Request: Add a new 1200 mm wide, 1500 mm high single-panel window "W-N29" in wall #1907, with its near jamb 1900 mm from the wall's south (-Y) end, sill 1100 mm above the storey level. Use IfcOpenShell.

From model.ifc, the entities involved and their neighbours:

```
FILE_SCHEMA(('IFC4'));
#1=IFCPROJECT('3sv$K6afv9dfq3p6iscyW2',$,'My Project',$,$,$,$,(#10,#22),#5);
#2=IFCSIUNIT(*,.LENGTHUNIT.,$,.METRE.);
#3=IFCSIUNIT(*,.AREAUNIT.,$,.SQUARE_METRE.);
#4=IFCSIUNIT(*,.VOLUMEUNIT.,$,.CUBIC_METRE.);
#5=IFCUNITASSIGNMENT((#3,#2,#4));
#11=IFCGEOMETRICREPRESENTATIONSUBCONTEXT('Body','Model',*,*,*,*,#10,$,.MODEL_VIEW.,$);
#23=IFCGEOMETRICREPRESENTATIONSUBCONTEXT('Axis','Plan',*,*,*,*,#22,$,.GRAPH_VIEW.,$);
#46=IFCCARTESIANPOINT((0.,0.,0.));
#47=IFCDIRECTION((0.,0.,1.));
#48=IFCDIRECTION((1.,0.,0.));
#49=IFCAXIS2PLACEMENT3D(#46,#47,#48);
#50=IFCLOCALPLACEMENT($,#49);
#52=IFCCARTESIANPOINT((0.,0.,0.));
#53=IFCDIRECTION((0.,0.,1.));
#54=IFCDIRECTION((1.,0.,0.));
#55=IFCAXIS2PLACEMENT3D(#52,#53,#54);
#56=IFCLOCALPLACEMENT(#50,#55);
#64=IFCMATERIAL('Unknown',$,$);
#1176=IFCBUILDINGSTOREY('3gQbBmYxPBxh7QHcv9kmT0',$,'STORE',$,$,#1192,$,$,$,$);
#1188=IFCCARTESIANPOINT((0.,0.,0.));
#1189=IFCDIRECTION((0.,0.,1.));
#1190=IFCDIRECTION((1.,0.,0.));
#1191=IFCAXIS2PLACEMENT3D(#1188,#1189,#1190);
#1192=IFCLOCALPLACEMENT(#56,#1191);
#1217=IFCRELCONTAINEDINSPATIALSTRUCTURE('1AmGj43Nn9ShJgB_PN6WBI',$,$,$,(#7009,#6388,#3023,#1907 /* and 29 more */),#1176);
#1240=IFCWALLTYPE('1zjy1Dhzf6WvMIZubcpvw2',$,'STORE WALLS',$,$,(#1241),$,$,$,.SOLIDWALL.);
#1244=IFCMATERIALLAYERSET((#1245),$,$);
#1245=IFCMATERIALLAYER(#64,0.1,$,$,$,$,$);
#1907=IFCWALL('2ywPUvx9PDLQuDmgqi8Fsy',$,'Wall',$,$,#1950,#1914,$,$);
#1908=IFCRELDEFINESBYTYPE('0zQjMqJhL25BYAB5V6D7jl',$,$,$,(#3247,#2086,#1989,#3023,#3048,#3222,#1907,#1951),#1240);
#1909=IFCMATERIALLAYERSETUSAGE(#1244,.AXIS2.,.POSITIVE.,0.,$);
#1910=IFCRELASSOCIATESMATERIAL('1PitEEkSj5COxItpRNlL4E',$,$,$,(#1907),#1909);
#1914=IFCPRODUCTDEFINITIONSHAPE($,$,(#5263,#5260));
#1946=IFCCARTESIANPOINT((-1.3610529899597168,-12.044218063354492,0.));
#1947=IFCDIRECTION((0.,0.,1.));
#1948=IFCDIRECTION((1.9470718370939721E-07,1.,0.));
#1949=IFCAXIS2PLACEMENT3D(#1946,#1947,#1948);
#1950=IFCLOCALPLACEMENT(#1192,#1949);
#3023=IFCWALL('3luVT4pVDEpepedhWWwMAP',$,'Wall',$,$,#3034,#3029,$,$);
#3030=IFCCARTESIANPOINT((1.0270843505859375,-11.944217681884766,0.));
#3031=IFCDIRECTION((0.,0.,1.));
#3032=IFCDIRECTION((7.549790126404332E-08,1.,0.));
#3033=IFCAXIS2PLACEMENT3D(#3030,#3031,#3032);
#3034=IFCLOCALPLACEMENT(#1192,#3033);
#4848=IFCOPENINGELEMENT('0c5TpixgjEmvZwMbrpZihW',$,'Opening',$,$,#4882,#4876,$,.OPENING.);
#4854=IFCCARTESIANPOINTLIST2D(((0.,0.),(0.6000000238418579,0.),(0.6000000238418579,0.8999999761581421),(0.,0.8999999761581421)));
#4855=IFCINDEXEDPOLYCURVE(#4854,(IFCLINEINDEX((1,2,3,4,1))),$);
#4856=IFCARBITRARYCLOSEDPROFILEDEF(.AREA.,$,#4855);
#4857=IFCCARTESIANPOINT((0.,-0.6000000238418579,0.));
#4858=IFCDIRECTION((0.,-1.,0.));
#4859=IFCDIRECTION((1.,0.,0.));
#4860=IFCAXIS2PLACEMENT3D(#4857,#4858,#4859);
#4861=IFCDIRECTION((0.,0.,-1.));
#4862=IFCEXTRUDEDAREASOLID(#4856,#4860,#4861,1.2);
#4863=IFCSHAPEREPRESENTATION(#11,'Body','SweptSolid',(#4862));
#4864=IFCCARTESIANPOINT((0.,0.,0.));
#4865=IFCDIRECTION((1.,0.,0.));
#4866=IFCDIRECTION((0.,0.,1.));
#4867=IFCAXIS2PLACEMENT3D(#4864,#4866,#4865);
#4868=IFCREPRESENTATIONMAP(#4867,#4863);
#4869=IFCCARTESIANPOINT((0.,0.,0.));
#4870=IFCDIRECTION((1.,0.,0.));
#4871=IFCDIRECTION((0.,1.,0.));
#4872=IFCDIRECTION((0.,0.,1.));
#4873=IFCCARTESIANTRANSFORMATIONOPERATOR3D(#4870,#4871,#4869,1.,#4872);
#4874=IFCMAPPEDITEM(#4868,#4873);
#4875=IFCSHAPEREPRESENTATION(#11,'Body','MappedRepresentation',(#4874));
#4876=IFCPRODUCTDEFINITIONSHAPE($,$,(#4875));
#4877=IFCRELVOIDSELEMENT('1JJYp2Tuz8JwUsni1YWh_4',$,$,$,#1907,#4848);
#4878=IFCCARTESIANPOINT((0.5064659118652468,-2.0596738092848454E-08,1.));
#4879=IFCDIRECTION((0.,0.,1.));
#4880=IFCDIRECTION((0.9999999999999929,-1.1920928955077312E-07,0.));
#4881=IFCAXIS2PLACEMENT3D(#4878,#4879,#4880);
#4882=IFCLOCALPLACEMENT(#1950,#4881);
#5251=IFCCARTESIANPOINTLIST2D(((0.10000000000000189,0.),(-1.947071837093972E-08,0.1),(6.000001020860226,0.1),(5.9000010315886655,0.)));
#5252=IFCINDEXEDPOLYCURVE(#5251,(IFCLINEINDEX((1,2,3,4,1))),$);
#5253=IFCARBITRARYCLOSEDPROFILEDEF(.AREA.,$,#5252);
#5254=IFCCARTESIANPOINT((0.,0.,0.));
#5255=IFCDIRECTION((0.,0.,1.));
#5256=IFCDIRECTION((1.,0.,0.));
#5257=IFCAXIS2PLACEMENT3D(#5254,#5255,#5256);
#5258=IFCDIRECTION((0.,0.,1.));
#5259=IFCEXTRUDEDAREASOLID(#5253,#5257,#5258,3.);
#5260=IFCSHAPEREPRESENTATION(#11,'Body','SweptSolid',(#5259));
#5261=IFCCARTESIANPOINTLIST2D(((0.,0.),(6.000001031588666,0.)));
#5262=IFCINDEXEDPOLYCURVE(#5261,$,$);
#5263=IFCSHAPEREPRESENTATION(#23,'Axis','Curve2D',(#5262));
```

```python
import numpy as np
import ifcopenshell
import ifcopenshell.api.feature
import ifcopenshell.api.geometry
import ifcopenshell.api.root
import ifcopenshell.api.spatial
import ifcopenshell.geom
import ifcopenshell.util.element
import ifcopenshell.util.placement
import ifcopenshell.util.representation
import ifcopenshell.util.shape
import ifcopenshell.util.unit

model = ifcopenshell.open("model.ifc")
unit_scale = ifcopenshell.util.unit.calculate_unit_scale(model)
settings = ifcopenshell.geom.settings()


def volume(element):
    """Net volume in cubic metres, openings subtracted."""
    shape = ifcopenshell.geom.create_shape(settings, element)
    return ifcopenshell.util.shape.get_volume(shape.geometry)


wall = model.by_guid("2ywPUvx9PDLQuDmgqi8Fsy")
storey = ifcopenshell.util.element.get_container(wall, ifc_class="IfcBuildingStorey")
context = ifcopenshell.util.representation.get_context(model, "Model", "Body", "MODEL_VIEW")
before = volume(wall)

width, height, from_end, sill = 1.2, 1.5, 1.9, 1.1  # metres

# The wall runs along its own X axis, and the end named is its -X end.
wall_shape = ifcopenshell.geom.create_shape(settings, wall)
x, y, z = ifcopenshell.util.shape.get_vertices(wall_shape.geometry).T
start = x.min() + from_end
face, thickness = float(y.min()), float(y.max() - y.min())
wall_matrix = ifcopenshell.util.placement.get_local_placement(wall.ObjectPlacement)
level = ifcopenshell.util.placement.get_local_placement(storey.ObjectPlacement)[2, 3]


def in_wall(x, y):
    """Placement at x, y metres in the wall's axes, at sill height."""
    matrix = wall_matrix.copy()
    matrix[:, 3] = wall_matrix @ np.array([x / unit_scale, y / unit_scale, 0.0, 1.0])
    matrix[2, 3] = level + sill / unit_scale
    return matrix


# Opening: a box that overshoots both wall faces by 50 mm.
opening = ifcopenshell.api.root.create_entity(model, ifc_class="IfcOpeningElement", predefined_type="OPENING")
box = ifcopenshell.api.geometry.add_wall_representation(
    model, context=context, length=width, height=height, thickness=thickness + 0.1
)
ifcopenshell.api.geometry.assign_representation(model, product=opening, representation=box)
ifcopenshell.api.geometry.edit_object_placement(model, product=opening, matrix=in_wall(start, face - 0.05), is_si=False)
ifcopenshell.api.feature.add_feature(model, feature=opening, element=wall)

window = ifcopenshell.api.root.create_entity(model, ifc_class="IfcWindow", name="W-N29", predefined_type="WINDOW")
window.OverallWidth, window.OverallHeight = width / unit_scale, height / unit_scale
window.PartitioningType = "SINGLE_PANEL"
body = ifcopenshell.api.geometry.add_window_representation(
    model,
    context=context,
    overall_width=window.OverallWidth,
    overall_height=window.OverallHeight,
    partition_type="SINGLE_PANEL",
)
ifcopenshell.api.geometry.assign_representation(model, product=window, representation=body)
ifcopenshell.api.spatial.assign_container(model, products=[window], relating_structure=storey)
ifcopenshell.api.feature.add_filling(model, opening=opening, element=window)

# Centre the window in the wall's thickness.
ifcopenshell.api.geometry.edit_object_placement(model, product=window, matrix=in_wall(start, face), is_si=False)
window_shape = ifcopenshell.geom.create_shape(settings, window)
depth = ifcopenshell.util.shape.get_vertices(window_shape.geometry)[:, 1]
offset = face + thickness / 2 - (depth.min() + depth.max()) / 2
ifcopenshell.api.geometry.edit_object_placement(model, product=window, matrix=in_wall(start, offset), is_si=False)

after = volume(wall)

print(f"wall volume {before:.3f} -> {after:.3f} m3")

model.write("model_updated.ifc")
```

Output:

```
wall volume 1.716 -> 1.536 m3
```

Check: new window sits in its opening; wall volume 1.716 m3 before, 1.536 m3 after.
